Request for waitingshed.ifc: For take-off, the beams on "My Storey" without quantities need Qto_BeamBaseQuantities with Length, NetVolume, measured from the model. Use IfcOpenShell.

First a look at what the model holds.

```python
import ifcopenshell
import ifcopenshell.util.element
import ifcopenshell.util.unit

model = ifcopenshell.open("waitingshed.ifc")
print(model.schema)
for unit_type in ("LENGTHUNIT", "AREAUNIT", "VOLUMEUNIT"):
    print(unit_type, ifcopenshell.util.unit.calculate_unit_scale(model, unit_type))
storey = next(s for s in model.by_type("IfcBuildingStorey") if s.Name == "My Storey")
beams = [e for e in ifcopenshell.util.element.get_decomposition(storey) if e.is_a("IfcBeam")]
for e in sorted(beams, key=lambda e: e.id()):
    print(e.id(), e.is_a(), e.Name, list(ifcopenshell.util.element.get_psets(e, qtos_only=True)), sep=" | ")
```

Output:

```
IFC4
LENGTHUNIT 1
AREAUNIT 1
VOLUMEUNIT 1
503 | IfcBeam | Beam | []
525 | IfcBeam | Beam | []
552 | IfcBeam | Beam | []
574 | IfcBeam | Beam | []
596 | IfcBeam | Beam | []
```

```python
import ifcopenshell
import ifcopenshell.api.pset
import ifcopenshell.geom
import ifcopenshell.util.element
import ifcopenshell.util.shape
import ifcopenshell.util.unit

model = ifcopenshell.open("waitingshed.ifc")
unit_scale = ifcopenshell.util.unit.calculate_unit_scale(model)
volume_scale = ifcopenshell.util.unit.calculate_unit_scale(model, "VOLUMEUNIT")
settings = ifcopenshell.geom.settings()

storey = next(s for s in model.by_type("IfcBuildingStorey") if s.Name == "My Storey")
beams = [e for e in ifcopenshell.util.element.get_decomposition(storey) if e.is_a("IfcBeam")]

for e in sorted(beams, key=lambda e: e.id()):
    if ifcopenshell.util.element.get_psets(e, qtos_only=True, should_inherit=False):
        continue
    # Geometry comes back in metres, in the element's own axes.
    shape = ifcopenshell.geom.create_shape(settings, e)
    values = {
        "Length": ifcopenshell.util.shape.get_max_xyz(shape.geometry) / unit_scale,
        "NetVolume": ifcopenshell.util.shape.get_volume(shape.geometry) / volume_scale,
    }
    qto = ifcopenshell.api.pset.add_qto(model, product=e, name="Qto_BeamBaseQuantities")
    ifcopenshell.api.pset.edit_qto(model, qto=qto, properties=values)
    print(e.id(), {k: round(v, 3) for k, v in values.items()})

model.write("waitingshed_updated.ifc")
```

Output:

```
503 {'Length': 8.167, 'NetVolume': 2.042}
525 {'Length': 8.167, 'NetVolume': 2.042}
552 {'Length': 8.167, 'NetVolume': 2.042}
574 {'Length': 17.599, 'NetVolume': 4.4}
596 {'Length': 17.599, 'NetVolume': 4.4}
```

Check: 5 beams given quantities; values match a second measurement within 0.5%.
